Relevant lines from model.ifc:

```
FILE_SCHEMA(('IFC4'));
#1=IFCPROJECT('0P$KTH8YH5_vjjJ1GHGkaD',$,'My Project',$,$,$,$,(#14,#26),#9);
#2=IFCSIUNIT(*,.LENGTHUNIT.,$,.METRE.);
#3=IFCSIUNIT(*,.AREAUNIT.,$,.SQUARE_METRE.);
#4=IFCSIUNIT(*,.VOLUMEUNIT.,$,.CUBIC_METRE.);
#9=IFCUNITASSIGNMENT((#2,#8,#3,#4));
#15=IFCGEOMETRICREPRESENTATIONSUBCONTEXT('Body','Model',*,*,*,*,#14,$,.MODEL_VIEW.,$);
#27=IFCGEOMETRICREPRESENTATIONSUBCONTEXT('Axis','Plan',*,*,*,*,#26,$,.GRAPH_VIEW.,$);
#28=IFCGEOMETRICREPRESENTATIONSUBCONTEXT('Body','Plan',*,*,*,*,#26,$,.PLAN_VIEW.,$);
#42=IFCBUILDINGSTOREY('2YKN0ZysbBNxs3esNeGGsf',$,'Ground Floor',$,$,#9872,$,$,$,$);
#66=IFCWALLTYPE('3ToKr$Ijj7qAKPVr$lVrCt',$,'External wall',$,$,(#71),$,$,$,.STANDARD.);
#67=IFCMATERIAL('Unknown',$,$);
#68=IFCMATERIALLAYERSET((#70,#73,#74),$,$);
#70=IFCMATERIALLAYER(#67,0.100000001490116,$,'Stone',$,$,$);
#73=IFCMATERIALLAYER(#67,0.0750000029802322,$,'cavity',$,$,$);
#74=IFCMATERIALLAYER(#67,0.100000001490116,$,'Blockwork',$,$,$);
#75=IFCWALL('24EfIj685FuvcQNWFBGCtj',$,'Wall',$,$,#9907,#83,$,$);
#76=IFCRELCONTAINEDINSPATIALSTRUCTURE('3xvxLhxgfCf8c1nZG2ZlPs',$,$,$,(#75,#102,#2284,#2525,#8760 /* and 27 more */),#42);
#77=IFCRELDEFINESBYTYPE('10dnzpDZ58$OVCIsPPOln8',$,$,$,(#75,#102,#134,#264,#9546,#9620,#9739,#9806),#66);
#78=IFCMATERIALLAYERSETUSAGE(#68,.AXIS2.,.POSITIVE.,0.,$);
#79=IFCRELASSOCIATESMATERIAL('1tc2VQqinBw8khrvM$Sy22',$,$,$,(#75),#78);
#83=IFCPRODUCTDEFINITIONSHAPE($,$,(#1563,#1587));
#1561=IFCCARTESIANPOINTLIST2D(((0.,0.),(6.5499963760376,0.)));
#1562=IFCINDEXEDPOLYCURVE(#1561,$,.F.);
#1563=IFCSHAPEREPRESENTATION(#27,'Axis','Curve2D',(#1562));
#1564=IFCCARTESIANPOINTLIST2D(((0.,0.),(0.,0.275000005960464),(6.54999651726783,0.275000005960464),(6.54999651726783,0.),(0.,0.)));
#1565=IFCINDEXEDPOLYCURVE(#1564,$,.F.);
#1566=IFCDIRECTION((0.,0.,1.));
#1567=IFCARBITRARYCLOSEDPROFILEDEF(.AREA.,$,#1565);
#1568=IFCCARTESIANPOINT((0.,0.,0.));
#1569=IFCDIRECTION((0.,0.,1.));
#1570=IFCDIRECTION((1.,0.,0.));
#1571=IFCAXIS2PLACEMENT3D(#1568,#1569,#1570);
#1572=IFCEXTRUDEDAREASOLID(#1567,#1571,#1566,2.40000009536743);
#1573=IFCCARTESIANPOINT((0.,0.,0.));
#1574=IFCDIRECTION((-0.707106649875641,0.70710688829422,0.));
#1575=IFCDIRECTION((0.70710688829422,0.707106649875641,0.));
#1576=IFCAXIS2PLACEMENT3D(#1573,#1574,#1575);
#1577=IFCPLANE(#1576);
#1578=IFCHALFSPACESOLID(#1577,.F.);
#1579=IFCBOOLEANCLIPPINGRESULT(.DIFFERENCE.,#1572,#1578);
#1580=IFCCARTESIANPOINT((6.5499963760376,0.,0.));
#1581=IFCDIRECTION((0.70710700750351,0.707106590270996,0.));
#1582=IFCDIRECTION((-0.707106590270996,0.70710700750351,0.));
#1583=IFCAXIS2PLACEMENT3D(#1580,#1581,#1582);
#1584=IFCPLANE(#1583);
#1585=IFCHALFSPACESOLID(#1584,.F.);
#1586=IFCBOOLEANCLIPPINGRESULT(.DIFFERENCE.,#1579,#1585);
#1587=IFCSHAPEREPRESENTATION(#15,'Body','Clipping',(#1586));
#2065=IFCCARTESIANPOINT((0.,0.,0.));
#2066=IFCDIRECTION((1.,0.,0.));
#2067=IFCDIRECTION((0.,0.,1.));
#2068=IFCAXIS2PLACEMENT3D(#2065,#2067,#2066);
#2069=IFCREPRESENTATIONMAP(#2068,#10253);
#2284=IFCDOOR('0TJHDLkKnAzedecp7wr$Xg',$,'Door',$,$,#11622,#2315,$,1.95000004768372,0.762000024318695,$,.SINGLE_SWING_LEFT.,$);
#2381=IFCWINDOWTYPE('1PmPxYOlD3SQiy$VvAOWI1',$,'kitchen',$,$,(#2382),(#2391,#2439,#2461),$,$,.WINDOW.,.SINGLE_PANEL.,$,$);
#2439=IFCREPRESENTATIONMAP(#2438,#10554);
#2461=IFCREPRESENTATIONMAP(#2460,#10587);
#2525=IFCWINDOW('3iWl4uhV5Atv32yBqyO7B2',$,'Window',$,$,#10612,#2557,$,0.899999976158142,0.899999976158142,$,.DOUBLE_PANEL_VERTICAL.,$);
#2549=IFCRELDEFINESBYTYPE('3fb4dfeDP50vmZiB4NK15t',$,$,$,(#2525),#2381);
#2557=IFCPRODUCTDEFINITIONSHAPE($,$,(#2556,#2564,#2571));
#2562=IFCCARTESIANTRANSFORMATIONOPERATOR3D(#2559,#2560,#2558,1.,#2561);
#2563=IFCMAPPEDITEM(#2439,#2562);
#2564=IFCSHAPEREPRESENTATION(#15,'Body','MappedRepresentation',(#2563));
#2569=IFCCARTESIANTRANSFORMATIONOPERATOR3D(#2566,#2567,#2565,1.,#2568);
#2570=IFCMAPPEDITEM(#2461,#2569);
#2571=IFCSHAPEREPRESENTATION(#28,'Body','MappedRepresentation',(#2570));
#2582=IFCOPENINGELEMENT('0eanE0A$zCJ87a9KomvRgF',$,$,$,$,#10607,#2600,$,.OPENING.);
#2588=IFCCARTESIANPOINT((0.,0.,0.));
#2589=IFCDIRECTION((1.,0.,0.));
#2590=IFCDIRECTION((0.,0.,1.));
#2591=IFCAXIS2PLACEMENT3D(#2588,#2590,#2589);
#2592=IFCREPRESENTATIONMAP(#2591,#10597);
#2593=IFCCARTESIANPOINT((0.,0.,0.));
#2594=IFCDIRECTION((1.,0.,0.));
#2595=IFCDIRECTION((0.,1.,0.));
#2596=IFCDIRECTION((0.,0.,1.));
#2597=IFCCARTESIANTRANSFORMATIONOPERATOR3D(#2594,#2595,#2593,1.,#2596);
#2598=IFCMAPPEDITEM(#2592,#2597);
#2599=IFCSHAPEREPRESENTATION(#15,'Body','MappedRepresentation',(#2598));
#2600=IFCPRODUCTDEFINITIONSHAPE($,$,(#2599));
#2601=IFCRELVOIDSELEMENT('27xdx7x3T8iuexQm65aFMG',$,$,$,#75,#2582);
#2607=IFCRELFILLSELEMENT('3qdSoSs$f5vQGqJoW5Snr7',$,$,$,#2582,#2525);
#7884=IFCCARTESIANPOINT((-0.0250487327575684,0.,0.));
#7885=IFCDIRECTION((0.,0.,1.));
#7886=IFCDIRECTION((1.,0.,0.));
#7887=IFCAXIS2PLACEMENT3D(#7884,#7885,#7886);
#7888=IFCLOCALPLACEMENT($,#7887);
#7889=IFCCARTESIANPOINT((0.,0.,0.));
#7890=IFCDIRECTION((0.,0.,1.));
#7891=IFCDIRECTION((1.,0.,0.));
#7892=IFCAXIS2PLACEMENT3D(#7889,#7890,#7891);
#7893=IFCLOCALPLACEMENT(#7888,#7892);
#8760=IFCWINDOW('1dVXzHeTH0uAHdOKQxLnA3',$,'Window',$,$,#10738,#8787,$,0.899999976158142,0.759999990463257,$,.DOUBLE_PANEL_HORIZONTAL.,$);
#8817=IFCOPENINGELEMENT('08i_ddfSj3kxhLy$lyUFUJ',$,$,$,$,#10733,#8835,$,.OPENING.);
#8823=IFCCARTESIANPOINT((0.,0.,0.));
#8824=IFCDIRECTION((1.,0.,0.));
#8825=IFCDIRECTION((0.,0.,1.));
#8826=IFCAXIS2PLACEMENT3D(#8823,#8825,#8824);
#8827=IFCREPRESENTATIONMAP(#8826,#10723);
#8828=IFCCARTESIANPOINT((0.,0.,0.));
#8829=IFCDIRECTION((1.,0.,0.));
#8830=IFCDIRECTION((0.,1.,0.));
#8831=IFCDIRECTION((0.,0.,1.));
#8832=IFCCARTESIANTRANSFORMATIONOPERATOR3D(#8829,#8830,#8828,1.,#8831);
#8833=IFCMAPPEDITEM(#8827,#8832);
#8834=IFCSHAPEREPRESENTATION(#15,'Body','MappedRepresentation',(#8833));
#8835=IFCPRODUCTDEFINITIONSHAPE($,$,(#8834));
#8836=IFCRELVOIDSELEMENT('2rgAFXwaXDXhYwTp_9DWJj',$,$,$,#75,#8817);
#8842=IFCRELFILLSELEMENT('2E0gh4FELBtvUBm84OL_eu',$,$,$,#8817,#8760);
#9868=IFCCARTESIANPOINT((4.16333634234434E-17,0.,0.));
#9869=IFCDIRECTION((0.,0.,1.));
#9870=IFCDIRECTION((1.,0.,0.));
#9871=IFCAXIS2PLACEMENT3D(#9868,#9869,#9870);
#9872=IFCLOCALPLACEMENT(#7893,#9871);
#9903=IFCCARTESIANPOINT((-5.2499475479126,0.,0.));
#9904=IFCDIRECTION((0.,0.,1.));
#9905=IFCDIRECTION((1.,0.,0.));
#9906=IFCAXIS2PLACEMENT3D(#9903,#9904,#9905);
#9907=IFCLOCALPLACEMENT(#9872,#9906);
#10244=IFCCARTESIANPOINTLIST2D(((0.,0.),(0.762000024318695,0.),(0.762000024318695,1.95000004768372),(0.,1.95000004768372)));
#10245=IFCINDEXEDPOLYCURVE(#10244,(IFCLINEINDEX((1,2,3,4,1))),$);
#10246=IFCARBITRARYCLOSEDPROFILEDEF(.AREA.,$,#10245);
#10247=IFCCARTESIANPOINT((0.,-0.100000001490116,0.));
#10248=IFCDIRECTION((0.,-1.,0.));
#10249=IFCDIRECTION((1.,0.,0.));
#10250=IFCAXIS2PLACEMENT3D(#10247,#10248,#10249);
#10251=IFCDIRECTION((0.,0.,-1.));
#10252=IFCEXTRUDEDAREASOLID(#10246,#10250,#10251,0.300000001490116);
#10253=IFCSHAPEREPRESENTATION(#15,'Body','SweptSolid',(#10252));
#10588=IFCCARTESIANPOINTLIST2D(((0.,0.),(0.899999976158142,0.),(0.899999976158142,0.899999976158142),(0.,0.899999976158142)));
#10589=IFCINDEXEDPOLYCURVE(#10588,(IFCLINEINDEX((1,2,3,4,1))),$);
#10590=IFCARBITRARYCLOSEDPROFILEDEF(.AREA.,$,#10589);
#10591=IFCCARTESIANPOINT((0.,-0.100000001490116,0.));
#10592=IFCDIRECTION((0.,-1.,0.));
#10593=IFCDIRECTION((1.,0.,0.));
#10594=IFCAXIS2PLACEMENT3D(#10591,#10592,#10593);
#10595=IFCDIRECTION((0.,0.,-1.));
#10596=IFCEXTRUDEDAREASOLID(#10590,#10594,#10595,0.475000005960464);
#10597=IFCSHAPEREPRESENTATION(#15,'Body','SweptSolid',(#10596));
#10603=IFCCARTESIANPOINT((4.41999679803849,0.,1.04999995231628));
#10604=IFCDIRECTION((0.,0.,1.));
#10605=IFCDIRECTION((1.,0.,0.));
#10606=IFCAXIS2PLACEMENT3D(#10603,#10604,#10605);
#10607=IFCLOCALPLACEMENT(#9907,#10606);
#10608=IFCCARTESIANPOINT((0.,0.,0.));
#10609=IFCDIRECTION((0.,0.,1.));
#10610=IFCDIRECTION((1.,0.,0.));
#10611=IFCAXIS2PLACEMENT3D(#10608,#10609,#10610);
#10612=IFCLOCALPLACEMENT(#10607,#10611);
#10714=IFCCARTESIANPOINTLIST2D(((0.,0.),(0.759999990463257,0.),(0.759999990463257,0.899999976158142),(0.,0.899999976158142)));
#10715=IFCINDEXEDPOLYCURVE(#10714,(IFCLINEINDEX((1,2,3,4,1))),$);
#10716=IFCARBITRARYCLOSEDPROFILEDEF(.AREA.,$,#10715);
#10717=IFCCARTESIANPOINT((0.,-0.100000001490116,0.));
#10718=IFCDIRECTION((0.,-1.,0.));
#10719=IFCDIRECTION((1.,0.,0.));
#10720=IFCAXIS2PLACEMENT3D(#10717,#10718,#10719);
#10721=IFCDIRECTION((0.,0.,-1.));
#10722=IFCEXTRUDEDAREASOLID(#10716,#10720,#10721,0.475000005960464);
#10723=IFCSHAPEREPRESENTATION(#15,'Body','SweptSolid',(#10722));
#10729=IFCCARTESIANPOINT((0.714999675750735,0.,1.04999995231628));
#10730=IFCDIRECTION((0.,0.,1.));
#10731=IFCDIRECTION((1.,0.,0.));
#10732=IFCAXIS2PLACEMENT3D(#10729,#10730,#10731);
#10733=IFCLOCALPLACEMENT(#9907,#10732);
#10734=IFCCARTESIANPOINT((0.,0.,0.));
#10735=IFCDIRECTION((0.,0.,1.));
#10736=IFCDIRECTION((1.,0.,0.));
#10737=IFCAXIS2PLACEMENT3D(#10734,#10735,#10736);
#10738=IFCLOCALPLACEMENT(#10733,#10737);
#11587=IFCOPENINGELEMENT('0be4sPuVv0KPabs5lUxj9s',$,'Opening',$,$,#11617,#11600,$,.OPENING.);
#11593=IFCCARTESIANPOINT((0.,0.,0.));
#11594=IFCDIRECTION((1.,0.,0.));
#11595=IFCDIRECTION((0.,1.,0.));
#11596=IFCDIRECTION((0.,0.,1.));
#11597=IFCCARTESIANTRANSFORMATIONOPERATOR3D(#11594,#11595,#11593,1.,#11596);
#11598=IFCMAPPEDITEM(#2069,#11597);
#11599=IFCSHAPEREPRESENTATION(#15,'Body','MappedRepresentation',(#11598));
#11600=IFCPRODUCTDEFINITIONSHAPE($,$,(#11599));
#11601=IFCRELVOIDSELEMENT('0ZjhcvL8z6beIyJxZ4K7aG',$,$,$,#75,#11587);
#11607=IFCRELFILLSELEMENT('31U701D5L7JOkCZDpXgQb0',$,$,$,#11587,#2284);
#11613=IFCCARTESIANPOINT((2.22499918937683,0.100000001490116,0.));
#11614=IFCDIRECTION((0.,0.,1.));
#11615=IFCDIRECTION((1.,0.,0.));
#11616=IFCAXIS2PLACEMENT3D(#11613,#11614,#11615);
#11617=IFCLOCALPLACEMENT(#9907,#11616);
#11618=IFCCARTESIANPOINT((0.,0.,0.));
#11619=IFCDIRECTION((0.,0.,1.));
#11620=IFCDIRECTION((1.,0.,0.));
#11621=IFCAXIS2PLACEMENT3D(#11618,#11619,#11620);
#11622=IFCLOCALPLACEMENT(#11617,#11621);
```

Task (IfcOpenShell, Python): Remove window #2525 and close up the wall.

```python
import ifcopenshell
import ifcopenshell.api.feature
import ifcopenshell.api.root
import ifcopenshell.geom
import ifcopenshell.util.shape

model = ifcopenshell.open("model.ifc")
settings = ifcopenshell.geom.settings()


def volume(element):
    """Net volume in cubic metres, openings subtracted."""
    shape = ifcopenshell.geom.create_shape(settings, element)
    return ifcopenshell.util.shape.get_volume(shape.geometry)


window = model.by_guid("3iWl4uhV5Atv32yBqyO7B2")
opening = window.FillsVoids[0].RelatingOpeningElement
wall = opening.VoidsElements[0].RelatingBuildingElement
before = volume(wall)

ifcopenshell.api.root.remove_product(model, product=window)
ifcopenshell.api.feature.remove_feature(model, feature=opening)

after = volume(wall)

print(f"wall volume {before:.3f} -> {after:.3f} m3")

model.write("model-out.ifc")
```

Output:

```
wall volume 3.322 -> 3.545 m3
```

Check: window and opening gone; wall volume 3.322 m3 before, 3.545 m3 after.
